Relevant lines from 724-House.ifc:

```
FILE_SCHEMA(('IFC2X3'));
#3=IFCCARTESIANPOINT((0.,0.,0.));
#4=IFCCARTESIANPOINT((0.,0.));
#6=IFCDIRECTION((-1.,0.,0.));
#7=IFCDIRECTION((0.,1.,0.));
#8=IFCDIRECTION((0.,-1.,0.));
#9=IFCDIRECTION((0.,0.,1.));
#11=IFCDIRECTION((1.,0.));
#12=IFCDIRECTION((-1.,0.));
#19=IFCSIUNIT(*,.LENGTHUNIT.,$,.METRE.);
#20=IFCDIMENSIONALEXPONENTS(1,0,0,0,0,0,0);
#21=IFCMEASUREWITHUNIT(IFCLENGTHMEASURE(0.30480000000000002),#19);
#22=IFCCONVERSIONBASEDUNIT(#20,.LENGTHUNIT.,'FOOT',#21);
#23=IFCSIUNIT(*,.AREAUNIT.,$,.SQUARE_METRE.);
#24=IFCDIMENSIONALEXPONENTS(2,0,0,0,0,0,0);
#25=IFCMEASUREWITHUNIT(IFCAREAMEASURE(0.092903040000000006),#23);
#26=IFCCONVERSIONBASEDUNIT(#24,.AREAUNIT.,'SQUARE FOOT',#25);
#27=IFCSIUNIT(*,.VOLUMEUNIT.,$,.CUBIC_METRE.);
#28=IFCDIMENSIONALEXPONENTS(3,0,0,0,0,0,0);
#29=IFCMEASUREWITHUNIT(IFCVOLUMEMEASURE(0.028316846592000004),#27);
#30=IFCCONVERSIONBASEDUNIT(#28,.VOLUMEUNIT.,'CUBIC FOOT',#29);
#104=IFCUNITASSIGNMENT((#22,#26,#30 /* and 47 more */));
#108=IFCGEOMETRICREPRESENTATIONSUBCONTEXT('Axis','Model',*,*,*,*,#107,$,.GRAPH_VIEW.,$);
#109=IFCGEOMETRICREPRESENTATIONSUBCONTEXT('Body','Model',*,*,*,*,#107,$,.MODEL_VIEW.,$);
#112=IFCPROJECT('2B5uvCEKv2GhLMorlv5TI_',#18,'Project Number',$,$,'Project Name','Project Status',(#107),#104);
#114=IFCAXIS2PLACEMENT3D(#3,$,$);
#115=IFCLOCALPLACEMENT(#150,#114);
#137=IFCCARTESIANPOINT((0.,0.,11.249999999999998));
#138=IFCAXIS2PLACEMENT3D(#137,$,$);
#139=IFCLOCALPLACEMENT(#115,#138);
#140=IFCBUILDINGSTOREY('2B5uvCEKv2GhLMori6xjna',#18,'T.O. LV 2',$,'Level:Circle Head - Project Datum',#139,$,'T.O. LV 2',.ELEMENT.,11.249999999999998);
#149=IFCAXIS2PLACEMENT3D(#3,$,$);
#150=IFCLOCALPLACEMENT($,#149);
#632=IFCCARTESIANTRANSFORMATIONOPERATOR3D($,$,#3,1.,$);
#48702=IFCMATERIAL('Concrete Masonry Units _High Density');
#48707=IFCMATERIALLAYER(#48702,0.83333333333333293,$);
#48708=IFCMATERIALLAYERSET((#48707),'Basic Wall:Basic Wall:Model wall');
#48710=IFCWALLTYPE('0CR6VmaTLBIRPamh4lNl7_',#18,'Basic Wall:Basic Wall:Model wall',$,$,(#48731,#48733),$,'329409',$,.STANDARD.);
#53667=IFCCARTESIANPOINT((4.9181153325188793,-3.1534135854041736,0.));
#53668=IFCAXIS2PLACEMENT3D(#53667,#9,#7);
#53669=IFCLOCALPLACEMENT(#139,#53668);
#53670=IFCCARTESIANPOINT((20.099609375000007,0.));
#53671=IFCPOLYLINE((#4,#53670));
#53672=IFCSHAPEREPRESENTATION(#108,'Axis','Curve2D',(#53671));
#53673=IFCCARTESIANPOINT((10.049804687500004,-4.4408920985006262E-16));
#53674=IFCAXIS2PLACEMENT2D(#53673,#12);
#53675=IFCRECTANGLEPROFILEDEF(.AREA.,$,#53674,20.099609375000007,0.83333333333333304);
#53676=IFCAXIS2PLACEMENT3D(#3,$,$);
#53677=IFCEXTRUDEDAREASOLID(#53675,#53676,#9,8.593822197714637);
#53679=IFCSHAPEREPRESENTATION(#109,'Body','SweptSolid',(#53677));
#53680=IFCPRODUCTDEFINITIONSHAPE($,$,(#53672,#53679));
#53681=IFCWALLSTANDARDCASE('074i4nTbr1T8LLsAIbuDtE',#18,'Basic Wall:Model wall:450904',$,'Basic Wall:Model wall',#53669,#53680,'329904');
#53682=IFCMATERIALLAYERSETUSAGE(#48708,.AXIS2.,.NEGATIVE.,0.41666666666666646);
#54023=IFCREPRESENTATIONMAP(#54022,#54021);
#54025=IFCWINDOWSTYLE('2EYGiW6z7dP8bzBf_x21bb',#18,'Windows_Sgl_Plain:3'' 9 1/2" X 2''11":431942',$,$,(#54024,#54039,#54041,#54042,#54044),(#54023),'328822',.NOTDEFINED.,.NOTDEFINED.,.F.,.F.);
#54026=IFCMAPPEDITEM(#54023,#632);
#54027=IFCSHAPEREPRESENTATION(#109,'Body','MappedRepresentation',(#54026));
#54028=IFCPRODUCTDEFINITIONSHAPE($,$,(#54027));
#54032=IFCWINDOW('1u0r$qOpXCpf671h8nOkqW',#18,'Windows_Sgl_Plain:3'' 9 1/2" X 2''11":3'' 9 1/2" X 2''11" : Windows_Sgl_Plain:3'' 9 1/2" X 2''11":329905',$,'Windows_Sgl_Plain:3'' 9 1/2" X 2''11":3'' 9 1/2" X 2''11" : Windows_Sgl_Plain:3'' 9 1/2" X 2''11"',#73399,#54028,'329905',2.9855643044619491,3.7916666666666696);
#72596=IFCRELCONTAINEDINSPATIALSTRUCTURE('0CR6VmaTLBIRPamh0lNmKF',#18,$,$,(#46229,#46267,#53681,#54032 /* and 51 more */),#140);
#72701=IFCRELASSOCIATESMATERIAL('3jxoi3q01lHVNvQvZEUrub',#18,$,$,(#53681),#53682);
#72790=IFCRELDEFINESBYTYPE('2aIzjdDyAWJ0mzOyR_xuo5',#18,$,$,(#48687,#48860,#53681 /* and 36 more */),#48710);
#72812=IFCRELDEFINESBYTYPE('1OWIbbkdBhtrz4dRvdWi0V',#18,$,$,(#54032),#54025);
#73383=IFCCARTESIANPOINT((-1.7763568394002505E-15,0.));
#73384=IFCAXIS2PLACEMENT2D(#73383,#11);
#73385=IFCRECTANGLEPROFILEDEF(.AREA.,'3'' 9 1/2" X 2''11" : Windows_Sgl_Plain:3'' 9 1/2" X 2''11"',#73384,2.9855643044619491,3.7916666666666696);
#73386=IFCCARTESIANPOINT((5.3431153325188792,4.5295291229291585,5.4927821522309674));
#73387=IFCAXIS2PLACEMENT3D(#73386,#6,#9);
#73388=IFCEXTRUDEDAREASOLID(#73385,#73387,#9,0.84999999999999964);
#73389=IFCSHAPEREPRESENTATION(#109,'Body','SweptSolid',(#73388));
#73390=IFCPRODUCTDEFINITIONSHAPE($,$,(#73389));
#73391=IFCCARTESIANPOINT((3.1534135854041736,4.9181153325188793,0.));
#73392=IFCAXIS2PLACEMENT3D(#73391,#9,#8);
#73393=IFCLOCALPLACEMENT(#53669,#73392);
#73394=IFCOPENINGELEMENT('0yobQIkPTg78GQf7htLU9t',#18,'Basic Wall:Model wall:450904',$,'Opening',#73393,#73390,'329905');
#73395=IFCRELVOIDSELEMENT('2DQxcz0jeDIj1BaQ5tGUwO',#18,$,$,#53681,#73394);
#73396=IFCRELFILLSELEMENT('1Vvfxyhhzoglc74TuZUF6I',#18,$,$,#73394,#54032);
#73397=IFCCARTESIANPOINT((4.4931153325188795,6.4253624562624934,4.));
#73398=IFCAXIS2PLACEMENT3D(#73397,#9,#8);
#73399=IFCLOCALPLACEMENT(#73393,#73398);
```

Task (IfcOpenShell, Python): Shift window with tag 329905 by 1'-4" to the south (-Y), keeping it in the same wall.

```python
import ifcopenshell
import ifcopenshell.api.geometry
import ifcopenshell.util.placement
import ifcopenshell.util.unit

model = ifcopenshell.open("724-House.ifc")
unit_scale = ifcopenshell.util.unit.calculate_unit_scale(model)

window = model.by_id(54032)
opening = window.FillsVoids[0].RelatingOpeningElement
wall = opening.VoidsElements[0].RelatingBuildingElement

wall_matrix = ifcopenshell.util.placement.get_local_placement(wall.ObjectPlacement)
shift = wall_matrix[:3, 0] * -16 * 0.0254 / unit_scale
before = ifcopenshell.util.placement.get_local_placement(window.ObjectPlacement)[:3, 3].copy()

# The window is placed relative to its opening, so it follows when the opening moves.
matrix = ifcopenshell.util.placement.get_local_placement(opening.ObjectPlacement)
matrix[:3, 3] += shift
ifcopenshell.api.geometry.edit_object_placement(
    model, product=opening, matrix=matrix, is_si=False, should_transform_children=True
)

after = ifcopenshell.util.placement.get_local_placement(window.ObjectPlacement)[:3, 3]
print("window moved by", (after - before).round(3) + 0.0)

model.write("724-House_v2.ifc")
```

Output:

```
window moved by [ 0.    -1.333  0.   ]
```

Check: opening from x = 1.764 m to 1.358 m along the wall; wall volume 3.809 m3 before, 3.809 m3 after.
